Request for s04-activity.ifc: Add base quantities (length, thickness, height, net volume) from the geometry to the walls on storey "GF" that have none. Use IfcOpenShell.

First a look at what the model holds.

```python
import ifcopenshell
import ifcopenshell.util.element
import ifcopenshell.util.unit

model = ifcopenshell.open("s04-activity.ifc")
print(model.schema)
for unit_type in ("LENGTHUNIT", "AREAUNIT", "VOLUMEUNIT"):
    print(unit_type, ifcopenshell.util.unit.calculate_unit_scale(model, unit_type))
storey = next(s for s in model.by_type("IfcBuildingStorey") if s.Name == "GF")
walls = [e for e in ifcopenshell.util.element.get_decomposition(storey) if e.is_a("IfcWall")]
for e in sorted(walls, key=lambda e: e.id()):
    print(e.id(), e.is_a(), e.Name, list(ifcopenshell.util.element.get_psets(e, qtos_only=True)), sep=" | ")
```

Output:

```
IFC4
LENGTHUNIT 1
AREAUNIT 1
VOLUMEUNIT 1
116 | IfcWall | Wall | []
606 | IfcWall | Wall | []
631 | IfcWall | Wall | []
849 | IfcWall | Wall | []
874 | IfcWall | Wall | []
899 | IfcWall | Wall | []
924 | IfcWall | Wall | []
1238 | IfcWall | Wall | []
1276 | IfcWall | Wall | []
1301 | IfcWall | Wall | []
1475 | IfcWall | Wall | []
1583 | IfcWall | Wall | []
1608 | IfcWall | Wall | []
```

```python
import ifcopenshell
import ifcopenshell.api.pset
import ifcopenshell.geom
import ifcopenshell.util.element
import ifcopenshell.util.shape
import ifcopenshell.util.unit

model = ifcopenshell.open("s04-activity.ifc")
unit_scale = ifcopenshell.util.unit.calculate_unit_scale(model)
volume_scale = ifcopenshell.util.unit.calculate_unit_scale(model, "VOLUMEUNIT")
settings = ifcopenshell.geom.settings()

storey = next(s for s in model.by_type("IfcBuildingStorey") if s.Name == "GF")
walls = [e for e in ifcopenshell.util.element.get_decomposition(storey) if e.is_a("IfcWall")]

for e in sorted(walls, key=lambda e: e.id()):
    if ifcopenshell.util.element.get_psets(e, qtos_only=True, should_inherit=False):
        continue
    # Geometry comes back in metres, in the element's own axes.
    shape = ifcopenshell.geom.create_shape(settings, e)
    values = {
        "Length": ifcopenshell.util.shape.get_x(shape.geometry) / unit_scale,
        "Width": ifcopenshell.util.shape.get_y(shape.geometry) / unit_scale,
        "Height": ifcopenshell.util.shape.get_z(shape.geometry) / unit_scale,
        "NetVolume": ifcopenshell.util.shape.get_volume(shape.geometry) / volume_scale,
    }
    qto = ifcopenshell.api.pset.add_qto(model, product=e, name="Qto_WallBaseQuantities")
    ifcopenshell.api.pset.edit_qto(model, qto=qto, properties=values)
    print(e.id(), {k: round(v, 3) for k, v in values.items()})

model.write("s04-activity_rev.ifc")
```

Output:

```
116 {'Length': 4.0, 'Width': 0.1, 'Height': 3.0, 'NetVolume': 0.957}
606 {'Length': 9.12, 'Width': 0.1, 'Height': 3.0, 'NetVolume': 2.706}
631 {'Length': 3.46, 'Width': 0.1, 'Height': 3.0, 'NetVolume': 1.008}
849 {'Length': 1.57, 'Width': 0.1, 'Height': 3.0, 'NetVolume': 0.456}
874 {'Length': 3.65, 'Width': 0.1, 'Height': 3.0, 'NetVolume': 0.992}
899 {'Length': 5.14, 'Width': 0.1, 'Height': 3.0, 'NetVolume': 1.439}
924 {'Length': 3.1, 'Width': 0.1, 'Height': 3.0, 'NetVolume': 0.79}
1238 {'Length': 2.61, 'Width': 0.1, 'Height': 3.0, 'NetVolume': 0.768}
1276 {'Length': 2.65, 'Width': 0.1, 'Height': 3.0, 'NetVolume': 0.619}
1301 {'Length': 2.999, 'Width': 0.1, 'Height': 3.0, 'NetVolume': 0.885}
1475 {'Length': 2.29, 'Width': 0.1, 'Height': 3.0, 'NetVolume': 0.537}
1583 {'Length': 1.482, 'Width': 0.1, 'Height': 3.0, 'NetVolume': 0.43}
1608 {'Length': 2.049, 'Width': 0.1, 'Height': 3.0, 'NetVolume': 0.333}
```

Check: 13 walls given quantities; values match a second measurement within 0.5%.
